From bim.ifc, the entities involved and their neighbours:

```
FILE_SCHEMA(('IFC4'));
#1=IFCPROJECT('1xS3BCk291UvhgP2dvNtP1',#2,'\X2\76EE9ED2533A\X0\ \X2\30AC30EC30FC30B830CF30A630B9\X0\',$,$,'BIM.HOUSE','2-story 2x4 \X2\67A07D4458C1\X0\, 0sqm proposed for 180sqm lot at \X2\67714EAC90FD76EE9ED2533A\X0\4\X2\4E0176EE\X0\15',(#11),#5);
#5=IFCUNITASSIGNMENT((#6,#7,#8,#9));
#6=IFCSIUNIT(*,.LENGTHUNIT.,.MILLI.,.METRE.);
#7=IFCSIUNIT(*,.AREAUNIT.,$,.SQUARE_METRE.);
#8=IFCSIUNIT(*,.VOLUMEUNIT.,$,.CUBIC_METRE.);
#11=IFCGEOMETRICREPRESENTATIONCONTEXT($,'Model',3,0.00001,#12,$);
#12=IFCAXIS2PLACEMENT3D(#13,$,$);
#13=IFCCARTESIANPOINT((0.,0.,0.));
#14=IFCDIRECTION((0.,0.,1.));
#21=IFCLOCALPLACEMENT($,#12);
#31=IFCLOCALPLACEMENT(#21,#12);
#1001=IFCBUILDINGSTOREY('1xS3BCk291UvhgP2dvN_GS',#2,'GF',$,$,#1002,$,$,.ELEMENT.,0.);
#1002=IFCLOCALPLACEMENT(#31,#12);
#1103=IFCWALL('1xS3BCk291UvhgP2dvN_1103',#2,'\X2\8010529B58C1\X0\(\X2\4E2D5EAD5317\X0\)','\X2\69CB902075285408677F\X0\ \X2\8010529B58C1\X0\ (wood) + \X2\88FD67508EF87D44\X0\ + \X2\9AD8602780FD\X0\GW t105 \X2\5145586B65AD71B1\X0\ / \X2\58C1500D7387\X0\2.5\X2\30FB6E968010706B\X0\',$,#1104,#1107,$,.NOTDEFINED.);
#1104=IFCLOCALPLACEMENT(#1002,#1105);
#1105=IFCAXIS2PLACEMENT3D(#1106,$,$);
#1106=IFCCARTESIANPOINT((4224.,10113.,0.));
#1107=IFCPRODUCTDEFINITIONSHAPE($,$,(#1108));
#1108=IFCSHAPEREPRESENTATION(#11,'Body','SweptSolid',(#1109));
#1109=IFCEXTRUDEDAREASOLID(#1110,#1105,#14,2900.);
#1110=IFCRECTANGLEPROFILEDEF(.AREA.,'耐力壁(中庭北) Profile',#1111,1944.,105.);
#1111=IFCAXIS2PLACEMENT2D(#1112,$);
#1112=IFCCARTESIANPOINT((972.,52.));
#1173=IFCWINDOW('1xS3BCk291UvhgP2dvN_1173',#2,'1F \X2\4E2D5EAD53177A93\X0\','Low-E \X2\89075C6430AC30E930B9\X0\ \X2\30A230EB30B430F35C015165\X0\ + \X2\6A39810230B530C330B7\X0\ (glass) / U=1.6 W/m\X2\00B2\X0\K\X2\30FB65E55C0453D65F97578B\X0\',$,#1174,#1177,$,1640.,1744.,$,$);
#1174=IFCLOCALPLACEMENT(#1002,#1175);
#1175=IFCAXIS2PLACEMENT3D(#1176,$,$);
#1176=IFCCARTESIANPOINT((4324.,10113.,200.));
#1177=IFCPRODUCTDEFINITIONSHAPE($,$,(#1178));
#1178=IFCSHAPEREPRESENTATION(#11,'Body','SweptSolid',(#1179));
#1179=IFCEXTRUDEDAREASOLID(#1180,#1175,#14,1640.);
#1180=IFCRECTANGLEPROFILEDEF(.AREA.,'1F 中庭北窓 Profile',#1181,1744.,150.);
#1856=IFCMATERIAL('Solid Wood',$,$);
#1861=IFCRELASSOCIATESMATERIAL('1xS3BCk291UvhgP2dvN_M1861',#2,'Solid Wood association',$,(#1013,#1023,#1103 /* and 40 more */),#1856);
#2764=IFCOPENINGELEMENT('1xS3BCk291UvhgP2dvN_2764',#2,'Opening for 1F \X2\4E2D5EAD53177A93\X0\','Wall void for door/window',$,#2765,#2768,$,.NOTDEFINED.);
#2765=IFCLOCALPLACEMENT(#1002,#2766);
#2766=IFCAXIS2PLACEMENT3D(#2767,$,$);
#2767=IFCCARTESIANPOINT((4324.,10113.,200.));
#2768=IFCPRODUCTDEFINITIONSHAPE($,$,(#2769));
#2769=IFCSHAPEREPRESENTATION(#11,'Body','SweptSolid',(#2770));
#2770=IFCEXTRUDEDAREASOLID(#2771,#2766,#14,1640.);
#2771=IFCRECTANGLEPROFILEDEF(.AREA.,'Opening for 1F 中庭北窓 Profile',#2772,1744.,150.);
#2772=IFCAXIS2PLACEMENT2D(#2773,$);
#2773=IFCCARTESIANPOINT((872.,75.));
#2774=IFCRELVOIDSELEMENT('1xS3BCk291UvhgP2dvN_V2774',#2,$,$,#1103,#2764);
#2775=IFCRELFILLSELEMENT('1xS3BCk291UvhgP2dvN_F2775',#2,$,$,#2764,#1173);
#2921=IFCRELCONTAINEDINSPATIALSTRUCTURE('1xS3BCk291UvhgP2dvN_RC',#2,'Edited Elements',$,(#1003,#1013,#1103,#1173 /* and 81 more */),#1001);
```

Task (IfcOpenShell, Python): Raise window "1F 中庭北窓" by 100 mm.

```python
import numpy as np
import ifcopenshell
import ifcopenshell.api.geometry
import ifcopenshell.util.placement
import ifcopenshell.util.unit

model = ifcopenshell.open("bim.ifc")
unit_scale = ifcopenshell.util.unit.calculate_unit_scale(model)

window = model.by_id(1173)
opening = window.FillsVoids[0].RelatingOpeningElement
dz = 0.1 / unit_scale

shift = np.array([0.0, 0.0, dz])
# The window is not placed relative to its opening, so move both.
for product in (opening, window):
    matrix = ifcopenshell.util.placement.get_local_placement(product.ObjectPlacement)
    matrix[:3, 3] += shift
    ifcopenshell.api.geometry.edit_object_placement(model, product=product, matrix=matrix, is_si=False)

print(f"moved by {dz * unit_scale:+.3f} m")

model.write("bim_rev.ifc")
```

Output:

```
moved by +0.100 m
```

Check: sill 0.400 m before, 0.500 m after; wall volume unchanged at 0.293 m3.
